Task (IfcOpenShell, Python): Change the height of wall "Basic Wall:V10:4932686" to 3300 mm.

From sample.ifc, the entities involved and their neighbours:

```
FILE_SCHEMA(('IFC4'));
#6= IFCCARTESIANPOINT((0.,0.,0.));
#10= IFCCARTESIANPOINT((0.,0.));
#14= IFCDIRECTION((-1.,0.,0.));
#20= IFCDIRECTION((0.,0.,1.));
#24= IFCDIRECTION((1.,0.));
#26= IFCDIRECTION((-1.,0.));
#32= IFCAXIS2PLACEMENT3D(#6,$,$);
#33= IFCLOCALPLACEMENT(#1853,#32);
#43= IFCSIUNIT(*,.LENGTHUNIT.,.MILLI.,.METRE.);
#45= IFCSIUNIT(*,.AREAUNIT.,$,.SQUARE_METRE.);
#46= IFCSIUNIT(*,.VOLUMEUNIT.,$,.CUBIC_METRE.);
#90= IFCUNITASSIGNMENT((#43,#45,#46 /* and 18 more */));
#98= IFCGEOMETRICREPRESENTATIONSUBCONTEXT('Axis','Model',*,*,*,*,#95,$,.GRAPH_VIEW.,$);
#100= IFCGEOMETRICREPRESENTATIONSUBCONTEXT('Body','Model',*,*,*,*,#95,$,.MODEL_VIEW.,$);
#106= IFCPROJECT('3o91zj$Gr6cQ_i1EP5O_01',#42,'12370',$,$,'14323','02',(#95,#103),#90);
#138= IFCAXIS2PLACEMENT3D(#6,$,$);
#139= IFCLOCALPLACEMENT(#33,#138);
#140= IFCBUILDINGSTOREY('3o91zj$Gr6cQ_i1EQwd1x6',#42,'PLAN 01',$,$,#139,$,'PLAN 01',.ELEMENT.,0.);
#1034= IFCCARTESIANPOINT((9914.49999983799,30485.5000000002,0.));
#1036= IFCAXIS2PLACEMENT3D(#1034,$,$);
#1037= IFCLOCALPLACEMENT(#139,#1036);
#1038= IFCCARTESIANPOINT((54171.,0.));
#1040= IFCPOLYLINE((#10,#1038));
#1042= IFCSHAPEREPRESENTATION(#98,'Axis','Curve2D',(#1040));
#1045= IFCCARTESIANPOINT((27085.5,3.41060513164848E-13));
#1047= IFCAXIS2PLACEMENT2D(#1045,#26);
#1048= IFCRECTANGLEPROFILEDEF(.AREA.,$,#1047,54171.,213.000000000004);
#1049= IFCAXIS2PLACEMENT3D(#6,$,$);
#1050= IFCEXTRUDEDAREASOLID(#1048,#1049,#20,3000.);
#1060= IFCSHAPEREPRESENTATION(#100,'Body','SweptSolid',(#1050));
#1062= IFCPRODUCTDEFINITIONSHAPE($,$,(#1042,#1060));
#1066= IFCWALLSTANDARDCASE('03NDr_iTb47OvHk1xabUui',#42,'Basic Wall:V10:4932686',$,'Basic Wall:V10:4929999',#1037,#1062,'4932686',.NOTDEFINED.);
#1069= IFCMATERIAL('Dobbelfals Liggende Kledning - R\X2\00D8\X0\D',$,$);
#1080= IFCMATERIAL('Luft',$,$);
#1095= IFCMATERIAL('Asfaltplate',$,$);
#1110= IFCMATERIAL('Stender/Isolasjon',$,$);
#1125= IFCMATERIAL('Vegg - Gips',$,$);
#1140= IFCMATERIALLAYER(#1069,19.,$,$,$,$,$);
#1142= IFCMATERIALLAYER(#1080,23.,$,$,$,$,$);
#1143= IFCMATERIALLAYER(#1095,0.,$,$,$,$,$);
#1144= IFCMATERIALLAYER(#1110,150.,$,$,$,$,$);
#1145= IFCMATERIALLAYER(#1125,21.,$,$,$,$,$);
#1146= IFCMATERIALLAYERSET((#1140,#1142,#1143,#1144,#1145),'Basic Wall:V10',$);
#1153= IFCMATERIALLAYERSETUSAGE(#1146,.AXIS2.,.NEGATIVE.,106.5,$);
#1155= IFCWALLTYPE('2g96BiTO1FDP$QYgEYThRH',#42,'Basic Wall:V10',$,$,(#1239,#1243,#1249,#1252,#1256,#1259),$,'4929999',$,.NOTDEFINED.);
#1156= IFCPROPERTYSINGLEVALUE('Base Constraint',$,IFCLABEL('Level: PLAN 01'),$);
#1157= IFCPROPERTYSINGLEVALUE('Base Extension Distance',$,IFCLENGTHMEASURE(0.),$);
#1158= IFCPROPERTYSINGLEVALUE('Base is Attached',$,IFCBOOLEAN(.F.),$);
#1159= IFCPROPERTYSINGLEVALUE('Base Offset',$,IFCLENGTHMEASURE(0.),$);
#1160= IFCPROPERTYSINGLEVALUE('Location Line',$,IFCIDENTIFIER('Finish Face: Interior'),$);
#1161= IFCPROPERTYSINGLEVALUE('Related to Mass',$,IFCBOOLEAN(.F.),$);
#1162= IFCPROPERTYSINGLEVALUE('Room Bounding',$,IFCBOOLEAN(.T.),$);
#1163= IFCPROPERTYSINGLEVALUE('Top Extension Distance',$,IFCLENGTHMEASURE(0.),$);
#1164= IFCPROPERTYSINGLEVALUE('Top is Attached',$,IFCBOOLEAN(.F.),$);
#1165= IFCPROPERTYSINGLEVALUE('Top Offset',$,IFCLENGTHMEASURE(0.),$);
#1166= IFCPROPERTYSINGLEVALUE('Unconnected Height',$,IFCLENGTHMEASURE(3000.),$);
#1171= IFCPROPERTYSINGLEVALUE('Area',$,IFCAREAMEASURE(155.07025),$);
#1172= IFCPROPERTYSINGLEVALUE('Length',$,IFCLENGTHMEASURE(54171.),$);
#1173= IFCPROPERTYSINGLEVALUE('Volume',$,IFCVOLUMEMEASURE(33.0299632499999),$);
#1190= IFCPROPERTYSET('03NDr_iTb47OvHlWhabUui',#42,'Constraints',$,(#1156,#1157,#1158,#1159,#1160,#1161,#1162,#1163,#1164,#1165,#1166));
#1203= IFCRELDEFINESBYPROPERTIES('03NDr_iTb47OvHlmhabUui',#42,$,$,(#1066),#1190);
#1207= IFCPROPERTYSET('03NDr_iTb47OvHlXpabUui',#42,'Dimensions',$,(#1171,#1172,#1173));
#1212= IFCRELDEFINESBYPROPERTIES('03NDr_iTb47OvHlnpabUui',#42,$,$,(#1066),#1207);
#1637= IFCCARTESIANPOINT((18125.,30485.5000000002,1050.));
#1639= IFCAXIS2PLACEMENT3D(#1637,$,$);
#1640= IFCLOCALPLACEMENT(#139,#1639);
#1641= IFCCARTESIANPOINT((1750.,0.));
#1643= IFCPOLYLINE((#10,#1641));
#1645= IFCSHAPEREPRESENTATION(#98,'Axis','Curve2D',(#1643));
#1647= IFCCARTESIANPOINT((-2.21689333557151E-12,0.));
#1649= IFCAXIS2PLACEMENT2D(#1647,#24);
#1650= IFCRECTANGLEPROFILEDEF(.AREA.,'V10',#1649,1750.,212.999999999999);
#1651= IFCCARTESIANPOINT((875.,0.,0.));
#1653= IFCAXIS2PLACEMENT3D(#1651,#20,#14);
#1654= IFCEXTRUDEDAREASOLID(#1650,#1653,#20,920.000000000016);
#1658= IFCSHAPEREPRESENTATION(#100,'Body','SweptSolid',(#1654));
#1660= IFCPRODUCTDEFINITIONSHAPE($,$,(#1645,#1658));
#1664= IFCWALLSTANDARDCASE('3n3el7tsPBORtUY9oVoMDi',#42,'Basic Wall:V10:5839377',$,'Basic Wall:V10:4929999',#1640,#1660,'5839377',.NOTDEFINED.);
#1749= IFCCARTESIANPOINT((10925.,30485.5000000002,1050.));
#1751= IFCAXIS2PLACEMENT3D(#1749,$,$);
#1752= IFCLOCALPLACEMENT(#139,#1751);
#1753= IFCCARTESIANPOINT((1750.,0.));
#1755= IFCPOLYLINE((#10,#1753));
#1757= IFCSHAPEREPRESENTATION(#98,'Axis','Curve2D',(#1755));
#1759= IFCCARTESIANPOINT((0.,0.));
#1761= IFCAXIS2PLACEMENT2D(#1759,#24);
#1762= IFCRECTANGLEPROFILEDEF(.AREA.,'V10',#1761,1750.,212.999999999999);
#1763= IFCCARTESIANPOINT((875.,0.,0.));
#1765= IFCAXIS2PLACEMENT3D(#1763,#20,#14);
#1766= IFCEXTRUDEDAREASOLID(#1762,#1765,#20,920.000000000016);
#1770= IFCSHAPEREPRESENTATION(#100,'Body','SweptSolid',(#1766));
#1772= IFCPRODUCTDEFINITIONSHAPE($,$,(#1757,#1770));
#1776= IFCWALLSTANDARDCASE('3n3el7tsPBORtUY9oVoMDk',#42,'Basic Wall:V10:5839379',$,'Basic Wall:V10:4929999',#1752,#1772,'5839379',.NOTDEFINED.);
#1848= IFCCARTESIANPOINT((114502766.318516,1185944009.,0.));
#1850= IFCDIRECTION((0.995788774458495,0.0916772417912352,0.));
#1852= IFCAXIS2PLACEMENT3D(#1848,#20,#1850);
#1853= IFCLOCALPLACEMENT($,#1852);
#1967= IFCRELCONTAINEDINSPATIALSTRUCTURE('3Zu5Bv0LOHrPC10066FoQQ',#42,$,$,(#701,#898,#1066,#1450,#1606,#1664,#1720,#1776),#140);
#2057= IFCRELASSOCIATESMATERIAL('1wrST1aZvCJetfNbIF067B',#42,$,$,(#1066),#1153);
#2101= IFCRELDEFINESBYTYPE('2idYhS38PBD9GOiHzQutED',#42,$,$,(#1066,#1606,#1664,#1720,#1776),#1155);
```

```python
import ifcopenshell
import ifcopenshell.api.pset
import ifcopenshell.geom
import ifcopenshell.util.element
import ifcopenshell.util.representation
import ifcopenshell.util.shape
import ifcopenshell.util.unit

model = ifcopenshell.open("sample.ifc")
unit_scale = ifcopenshell.util.unit.calculate_unit_scale(model)
area_scale = ifcopenshell.util.unit.calculate_unit_scale(model, "AREAUNIT")
volume_scale = ifcopenshell.util.unit.calculate_unit_scale(model, "VOLUMEUNIT")
settings = ifcopenshell.geom.settings()


def volume(element):
    """Net volume in cubic metres, openings subtracted."""
    shape = ifcopenshell.geom.create_shape(settings, element)
    return ifcopenshell.util.shape.get_volume(shape.geometry)


wall = model.by_guid("03NDr_iTb47OvHk1xabUui")
before = volume(wall)

body = ifcopenshell.util.representation.get_representation(wall, "Model", "Body")
solid = body.Items[0]
old_height = solid.Depth
solid.Depth = 3.3 / unit_scale
after = volume(wall)
thickness = 0.213  # wall thickness in metres

# Update the stored height, areas and volumes.
pset = model.by_id(ifcopenshell.util.element.get_pset(wall, "Constraints", should_inherit=False)["id"])
ifcopenshell.api.pset.edit_pset(model, pset=pset, properties={
    "Unconnected Height": model.create_entity("IfcLengthMeasure", solid.Depth),
})
pset = model.by_id(ifcopenshell.util.element.get_pset(wall, "Dimensions", should_inherit=False)["id"])
ifcopenshell.api.pset.edit_pset(model, pset=pset, properties={
    "Area": model.create_entity("IfcAreaMeasure", after / thickness / area_scale),
    "Volume": model.create_entity("IfcVolumeMeasure", after / volume_scale),
})

print(f"height {old_height:g} -> {solid.Depth:g}, volume {before:.3f} -> {after:.3f} m3")

model.write("sample_updated.ifc")
```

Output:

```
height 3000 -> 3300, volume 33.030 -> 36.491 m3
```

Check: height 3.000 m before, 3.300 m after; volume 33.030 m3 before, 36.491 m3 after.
